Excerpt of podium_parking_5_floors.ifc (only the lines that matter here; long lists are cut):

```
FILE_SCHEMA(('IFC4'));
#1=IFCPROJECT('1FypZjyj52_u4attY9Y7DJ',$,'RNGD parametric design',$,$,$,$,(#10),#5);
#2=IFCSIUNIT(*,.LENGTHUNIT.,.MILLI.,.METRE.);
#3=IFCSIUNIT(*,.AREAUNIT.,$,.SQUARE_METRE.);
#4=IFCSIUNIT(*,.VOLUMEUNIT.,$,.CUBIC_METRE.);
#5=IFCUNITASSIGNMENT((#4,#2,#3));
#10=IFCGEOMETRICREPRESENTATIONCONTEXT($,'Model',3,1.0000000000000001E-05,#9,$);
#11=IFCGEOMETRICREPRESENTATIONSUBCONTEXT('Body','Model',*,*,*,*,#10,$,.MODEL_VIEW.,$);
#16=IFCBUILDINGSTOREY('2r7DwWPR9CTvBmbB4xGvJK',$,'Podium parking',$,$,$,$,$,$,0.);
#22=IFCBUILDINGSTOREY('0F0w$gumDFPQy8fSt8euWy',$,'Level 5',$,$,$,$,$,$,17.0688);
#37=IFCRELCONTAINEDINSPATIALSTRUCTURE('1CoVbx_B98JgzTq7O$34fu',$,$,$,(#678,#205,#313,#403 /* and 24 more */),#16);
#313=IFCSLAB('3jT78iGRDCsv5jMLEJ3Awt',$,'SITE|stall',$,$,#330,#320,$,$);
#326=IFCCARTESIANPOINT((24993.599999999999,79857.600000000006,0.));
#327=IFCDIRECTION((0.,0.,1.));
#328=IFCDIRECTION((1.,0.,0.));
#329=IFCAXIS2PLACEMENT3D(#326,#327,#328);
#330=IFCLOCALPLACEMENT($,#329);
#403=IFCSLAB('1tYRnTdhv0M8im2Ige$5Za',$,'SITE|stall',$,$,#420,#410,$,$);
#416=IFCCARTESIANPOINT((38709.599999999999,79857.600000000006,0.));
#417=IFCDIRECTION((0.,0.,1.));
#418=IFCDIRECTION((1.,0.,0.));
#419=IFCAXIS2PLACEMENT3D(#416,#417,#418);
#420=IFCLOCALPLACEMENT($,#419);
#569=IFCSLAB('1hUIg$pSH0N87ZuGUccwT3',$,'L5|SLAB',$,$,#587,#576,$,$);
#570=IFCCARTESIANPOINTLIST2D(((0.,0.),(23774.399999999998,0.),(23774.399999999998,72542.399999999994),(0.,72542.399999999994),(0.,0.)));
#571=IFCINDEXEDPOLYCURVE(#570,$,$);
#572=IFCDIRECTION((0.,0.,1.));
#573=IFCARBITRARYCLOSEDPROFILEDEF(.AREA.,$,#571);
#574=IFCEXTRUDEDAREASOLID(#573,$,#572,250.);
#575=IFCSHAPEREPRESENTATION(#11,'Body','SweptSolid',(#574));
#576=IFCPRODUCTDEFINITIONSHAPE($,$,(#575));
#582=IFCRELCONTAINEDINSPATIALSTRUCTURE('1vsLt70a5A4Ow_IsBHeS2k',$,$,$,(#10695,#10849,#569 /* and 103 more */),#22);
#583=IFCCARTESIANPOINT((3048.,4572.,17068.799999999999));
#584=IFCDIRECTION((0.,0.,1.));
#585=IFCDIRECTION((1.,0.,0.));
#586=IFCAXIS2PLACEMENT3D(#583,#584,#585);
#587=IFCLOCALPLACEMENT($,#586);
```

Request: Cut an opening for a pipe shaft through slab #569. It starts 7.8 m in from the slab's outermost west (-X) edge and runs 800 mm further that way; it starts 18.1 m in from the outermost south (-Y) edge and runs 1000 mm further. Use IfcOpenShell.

```python
import numpy as np
import ifcopenshell
import ifcopenshell.api.feature
import ifcopenshell.api.geometry
import ifcopenshell.api.root
import ifcopenshell.geom
import ifcopenshell.util.placement
import ifcopenshell.util.representation
import ifcopenshell.util.shape
import ifcopenshell.util.unit

model = ifcopenshell.open("podium_parking_5_floors.ifc")
unit_scale = ifcopenshell.util.unit.calculate_unit_scale(model)
settings = ifcopenshell.geom.settings()


def volume(element):
    """Net volume in cubic metres, openings subtracted."""
    shape = ifcopenshell.geom.create_shape(settings, element)
    return ifcopenshell.util.shape.get_volume(shape.geometry)


slab = model.by_id(569)
before = volume(slab)

# Extent in the slab's own axes, in metres. The edges named are its -X and -Y sides.
slab_shape = ifcopenshell.geom.create_shape(settings, slab)
vertices = ifcopenshell.util.shape.get_vertices(slab_shape.geometry)
x_min, y_min, bottom = vertices.min(axis=0)
top = vertices[:, 2].max()

opening = ifcopenshell.api.root.create_entity(model, ifc_class="IfcOpeningElement", name="Pipe shaft opening", predefined_type="OPENING")
context = ifcopenshell.util.representation.get_context(model, "Model", "Body", "MODEL_VIEW")
width, depth = 0.8, 1
outline = [(0.0, 0.0), (width, 0.0), (width, depth), (0.0, depth), (0.0, 0.0)]
# Overshoot both faces by 50 mm so the cut is clean.
shape = ifcopenshell.api.geometry.add_slab_representation(
    model, context=context, depth=top - bottom + 0.1, polyline=outline
)
ifcopenshell.api.geometry.assign_representation(model, product=opening, representation=shape)

matrix = ifcopenshell.util.placement.get_local_placement(slab.ObjectPlacement)
matrix[:, 3] = matrix @ np.append(np.array([x_min + 7.8, y_min + 18.1, bottom - 0.05]) / unit_scale, 1.0)
ifcopenshell.api.geometry.edit_object_placement(model, product=opening, matrix=matrix, is_si=False)
ifcopenshell.api.feature.add_feature(model, feature=opening, element=slab)

after = volume(slab)

print(f"slab volume {before:.3f} -> {after:.3f} m3")

model.write("podium_parking_5_floors_v2.ifc")
```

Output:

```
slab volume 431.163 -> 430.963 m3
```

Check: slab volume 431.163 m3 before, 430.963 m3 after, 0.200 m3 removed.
